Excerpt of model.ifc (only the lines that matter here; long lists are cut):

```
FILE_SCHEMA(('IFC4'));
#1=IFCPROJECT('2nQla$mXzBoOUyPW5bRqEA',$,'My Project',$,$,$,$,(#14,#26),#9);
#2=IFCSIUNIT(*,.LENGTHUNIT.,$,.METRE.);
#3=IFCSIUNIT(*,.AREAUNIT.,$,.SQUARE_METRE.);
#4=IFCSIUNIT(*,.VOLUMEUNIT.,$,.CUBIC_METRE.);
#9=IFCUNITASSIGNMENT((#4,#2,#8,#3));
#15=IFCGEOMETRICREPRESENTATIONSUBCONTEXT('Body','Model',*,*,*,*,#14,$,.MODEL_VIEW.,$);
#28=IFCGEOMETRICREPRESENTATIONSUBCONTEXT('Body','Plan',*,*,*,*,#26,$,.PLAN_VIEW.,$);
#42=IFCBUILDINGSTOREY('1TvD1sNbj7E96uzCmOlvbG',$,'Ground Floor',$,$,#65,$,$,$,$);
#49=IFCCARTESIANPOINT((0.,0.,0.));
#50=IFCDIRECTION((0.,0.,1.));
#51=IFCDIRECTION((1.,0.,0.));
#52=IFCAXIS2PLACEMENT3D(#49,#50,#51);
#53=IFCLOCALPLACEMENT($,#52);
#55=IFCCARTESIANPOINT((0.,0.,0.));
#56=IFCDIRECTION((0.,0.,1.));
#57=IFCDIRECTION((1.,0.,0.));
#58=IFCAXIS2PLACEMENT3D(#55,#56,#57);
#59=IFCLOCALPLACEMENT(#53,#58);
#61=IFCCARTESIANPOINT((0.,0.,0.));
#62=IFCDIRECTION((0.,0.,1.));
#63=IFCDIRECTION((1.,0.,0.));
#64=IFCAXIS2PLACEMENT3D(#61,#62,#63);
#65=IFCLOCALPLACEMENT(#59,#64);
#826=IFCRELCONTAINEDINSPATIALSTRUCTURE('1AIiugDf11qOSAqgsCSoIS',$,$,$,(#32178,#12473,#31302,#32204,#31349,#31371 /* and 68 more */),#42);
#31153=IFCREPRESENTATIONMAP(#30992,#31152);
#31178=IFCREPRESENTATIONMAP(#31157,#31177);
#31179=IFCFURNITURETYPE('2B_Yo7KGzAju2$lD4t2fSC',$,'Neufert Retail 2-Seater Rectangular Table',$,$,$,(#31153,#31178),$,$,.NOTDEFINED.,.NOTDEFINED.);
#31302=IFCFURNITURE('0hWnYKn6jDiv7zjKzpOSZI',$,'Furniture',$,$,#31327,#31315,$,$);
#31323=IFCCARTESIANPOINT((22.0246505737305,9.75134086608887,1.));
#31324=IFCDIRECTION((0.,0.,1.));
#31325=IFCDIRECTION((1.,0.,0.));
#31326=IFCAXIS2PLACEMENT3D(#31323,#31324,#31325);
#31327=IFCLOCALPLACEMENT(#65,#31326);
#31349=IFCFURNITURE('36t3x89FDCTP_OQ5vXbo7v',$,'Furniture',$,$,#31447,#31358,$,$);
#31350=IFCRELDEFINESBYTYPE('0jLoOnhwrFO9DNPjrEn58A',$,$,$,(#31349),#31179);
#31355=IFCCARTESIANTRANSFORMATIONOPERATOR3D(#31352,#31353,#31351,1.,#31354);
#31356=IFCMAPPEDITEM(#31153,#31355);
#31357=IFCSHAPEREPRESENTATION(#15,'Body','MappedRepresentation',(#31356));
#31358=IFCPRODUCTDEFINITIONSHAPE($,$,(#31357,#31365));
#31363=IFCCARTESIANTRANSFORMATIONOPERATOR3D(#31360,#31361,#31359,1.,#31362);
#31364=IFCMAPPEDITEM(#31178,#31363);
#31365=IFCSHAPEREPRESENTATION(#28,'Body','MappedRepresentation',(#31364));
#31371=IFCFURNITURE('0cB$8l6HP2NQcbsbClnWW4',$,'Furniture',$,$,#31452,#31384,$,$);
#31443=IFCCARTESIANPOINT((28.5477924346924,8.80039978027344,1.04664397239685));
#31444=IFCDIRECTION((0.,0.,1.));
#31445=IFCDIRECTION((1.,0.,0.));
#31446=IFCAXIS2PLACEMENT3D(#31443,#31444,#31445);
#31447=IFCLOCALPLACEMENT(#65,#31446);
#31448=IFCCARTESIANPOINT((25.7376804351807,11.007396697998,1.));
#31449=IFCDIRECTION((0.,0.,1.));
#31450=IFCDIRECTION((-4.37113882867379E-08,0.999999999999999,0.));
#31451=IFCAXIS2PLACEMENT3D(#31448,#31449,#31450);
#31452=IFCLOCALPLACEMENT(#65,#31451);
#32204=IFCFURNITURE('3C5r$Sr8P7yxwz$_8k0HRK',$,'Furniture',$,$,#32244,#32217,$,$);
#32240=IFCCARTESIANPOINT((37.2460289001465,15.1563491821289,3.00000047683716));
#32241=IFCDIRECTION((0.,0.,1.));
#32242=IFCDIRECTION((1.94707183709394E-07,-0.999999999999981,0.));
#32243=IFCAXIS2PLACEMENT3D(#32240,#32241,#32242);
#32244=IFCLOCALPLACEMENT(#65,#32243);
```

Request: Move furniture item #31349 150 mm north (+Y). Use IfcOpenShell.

```python
import ifcopenshell
import ifcopenshell.api.geometry
import ifcopenshell.util.placement

model = ifcopenshell.open("model.ifc")

item = model.by_id(31349)
matrix = ifcopenshell.util.placement.get_local_placement(item.ObjectPlacement)
matrix[1, 3] += 0.15
ifcopenshell.api.geometry.edit_object_placement(model, product=item, matrix=matrix, is_si=False)

print(ifcopenshell.util.placement.get_local_placement(item.ObjectPlacement).round(3) + 0.0)

model.write("model-out.ifc")
```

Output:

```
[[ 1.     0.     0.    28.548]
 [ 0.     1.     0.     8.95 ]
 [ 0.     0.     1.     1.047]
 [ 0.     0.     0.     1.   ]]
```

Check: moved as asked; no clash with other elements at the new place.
